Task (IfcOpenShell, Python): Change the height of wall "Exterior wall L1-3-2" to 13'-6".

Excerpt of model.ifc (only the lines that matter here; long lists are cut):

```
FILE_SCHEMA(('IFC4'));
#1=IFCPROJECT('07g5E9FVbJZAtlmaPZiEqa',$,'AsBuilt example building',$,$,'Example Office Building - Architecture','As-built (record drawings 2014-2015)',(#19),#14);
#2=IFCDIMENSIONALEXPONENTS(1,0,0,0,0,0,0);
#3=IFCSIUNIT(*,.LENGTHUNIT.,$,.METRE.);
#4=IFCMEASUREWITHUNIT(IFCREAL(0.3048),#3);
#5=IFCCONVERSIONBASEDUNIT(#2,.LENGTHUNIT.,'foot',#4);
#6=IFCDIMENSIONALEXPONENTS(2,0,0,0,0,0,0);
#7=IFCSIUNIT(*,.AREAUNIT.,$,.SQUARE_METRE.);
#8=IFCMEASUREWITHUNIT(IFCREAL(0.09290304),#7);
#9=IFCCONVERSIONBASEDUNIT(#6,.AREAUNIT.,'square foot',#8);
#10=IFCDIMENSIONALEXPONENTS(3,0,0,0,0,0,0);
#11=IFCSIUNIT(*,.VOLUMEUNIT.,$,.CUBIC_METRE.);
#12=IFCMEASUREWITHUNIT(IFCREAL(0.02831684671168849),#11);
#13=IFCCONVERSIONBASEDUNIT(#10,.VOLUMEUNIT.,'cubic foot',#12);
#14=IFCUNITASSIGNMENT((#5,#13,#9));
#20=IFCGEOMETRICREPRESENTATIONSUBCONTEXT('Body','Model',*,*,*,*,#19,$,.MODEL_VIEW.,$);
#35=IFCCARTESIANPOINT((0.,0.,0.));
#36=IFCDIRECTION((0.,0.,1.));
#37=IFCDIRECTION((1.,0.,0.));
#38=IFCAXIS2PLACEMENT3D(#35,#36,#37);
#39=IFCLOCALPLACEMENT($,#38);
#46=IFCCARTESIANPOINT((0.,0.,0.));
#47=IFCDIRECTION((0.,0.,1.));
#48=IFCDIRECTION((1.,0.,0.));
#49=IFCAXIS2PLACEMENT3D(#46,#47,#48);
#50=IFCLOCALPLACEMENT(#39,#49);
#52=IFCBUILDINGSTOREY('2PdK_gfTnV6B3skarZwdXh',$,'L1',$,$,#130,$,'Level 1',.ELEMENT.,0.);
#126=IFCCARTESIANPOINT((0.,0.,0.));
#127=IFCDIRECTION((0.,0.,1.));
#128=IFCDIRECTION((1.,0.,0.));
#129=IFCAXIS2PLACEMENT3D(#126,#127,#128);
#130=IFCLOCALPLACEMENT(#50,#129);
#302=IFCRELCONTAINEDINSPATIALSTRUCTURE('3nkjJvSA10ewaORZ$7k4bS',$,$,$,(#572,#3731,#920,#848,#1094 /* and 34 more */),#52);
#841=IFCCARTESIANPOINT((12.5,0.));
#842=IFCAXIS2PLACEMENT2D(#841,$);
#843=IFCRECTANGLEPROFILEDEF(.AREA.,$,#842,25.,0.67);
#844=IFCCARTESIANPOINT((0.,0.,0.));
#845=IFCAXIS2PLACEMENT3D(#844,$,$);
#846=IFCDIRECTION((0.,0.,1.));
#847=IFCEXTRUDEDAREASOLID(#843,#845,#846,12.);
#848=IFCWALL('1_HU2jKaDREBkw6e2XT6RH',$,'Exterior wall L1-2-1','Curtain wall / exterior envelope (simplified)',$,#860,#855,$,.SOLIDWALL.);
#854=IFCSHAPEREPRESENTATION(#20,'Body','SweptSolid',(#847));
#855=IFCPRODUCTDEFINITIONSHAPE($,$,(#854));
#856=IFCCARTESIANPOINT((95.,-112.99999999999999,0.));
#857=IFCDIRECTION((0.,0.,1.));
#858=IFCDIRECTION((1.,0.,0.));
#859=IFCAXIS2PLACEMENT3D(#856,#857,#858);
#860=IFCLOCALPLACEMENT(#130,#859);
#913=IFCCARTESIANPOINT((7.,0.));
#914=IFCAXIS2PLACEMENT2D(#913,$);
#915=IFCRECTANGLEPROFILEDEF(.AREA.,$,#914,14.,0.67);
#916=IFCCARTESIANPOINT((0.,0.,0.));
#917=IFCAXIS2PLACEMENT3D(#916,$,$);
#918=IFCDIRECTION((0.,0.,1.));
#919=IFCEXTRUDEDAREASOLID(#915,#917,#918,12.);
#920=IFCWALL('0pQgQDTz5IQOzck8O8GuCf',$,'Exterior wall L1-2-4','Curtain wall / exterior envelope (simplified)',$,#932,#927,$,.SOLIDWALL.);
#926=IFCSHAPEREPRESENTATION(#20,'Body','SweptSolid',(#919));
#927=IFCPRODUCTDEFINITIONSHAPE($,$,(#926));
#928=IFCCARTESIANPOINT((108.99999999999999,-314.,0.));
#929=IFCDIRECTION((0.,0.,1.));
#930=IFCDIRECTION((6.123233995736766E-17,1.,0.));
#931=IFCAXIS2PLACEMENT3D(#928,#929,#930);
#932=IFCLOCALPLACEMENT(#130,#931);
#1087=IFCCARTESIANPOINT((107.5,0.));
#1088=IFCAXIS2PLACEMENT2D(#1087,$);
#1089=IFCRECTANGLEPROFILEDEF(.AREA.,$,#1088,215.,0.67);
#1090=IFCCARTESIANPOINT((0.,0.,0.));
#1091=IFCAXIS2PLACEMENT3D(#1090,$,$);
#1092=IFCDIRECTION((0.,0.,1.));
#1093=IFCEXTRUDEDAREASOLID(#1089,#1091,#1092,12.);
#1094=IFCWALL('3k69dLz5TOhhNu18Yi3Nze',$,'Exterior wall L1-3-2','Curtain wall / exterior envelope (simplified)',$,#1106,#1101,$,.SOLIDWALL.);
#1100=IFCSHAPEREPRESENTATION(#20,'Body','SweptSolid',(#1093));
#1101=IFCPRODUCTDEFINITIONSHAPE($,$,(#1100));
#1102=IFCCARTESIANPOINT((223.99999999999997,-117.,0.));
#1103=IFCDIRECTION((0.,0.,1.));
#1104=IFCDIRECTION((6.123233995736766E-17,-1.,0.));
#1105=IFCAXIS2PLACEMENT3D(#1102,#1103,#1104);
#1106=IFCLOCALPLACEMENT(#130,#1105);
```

```python
import ifcopenshell
import ifcopenshell.geom
import ifcopenshell.util.representation
import ifcopenshell.util.shape
import ifcopenshell.util.unit

model = ifcopenshell.open("model.ifc")
unit_scale = ifcopenshell.util.unit.calculate_unit_scale(model)
settings = ifcopenshell.geom.settings()


def volume(element):
    """Net volume in cubic metres, openings subtracted."""
    shape = ifcopenshell.geom.create_shape(settings, element)
    return ifcopenshell.util.shape.get_volume(shape.geometry)


wall = model.by_id(1094)
before = volume(wall)

body = ifcopenshell.util.representation.get_representation(wall, "Model", "Body")
solid = body.Items[0]
old_height = solid.Depth
solid.Depth = 162 * 0.0254 / unit_scale
after = volume(wall)

print(f"height {old_height:g} -> {solid.Depth:g}, volume {before:.3f} -> {after:.3f} m3")

model.write("model_v2.ifc")
```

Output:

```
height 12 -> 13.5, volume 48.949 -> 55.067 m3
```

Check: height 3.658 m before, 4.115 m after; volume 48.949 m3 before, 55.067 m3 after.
